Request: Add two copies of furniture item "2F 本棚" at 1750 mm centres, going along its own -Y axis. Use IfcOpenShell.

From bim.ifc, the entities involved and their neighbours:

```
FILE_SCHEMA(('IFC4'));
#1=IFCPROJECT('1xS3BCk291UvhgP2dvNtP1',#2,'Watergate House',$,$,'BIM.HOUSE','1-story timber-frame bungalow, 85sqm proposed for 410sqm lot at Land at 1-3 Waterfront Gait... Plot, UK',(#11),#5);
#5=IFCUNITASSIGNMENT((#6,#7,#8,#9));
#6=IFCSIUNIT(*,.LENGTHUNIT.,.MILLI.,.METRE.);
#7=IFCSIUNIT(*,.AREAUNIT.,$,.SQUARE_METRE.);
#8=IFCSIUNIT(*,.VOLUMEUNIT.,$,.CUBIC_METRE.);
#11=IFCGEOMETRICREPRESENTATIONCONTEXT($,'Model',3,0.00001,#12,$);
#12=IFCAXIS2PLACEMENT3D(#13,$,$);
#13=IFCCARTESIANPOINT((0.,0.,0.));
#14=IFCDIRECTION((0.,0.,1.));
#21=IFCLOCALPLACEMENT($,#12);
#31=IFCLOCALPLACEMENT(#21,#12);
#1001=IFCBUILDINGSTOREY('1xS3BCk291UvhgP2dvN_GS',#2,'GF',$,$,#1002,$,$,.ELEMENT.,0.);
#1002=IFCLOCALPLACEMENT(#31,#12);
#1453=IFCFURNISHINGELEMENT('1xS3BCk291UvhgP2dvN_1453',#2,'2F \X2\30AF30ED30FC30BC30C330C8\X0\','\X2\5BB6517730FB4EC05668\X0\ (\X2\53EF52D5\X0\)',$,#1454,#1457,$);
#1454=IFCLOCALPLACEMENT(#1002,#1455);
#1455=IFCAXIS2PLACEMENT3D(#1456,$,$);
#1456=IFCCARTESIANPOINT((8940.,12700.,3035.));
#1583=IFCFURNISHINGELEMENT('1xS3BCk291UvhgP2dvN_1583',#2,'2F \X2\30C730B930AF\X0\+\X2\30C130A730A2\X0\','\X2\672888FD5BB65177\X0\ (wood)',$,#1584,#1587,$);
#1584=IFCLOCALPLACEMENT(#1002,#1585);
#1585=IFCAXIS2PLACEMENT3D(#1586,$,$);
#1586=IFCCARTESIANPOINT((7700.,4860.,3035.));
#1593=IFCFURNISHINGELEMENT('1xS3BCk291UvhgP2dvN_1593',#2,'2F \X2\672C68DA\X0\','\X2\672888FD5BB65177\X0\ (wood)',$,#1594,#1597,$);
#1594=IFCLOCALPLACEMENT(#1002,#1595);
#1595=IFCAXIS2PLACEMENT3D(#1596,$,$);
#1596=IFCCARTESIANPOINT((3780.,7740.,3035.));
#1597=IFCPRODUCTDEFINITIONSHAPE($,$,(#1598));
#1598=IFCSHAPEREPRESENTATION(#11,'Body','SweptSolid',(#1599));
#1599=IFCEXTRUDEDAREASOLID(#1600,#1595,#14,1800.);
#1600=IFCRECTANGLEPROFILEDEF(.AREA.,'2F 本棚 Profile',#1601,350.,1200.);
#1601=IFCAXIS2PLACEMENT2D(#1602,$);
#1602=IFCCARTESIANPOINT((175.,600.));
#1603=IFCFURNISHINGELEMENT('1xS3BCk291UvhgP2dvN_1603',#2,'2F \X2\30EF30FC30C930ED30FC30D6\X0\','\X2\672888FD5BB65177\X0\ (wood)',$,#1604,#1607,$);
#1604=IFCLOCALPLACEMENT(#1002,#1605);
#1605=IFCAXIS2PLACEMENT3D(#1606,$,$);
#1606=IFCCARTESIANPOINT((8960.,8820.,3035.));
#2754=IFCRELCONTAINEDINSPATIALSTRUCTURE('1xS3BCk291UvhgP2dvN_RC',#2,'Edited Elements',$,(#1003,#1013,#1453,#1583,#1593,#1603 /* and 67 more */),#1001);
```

```python
import ifcopenshell
import ifcopenshell.api.geometry
import ifcopenshell.api.root
import ifcopenshell.util.element
import ifcopenshell.util.placement
import ifcopenshell.util.unit

model = ifcopenshell.open("bim.ifc")
unit_scale = ifcopenshell.util.unit.calculate_unit_scale(model)


def reuse_history(source, copy):
    """copy_class also copies each property set's owner history, people and application; keep the originals."""
    for rel in copy.IsDefinedBy:
        if rel.is_a("IfcRelDefinesByProperties") and (history := rel.RelatingPropertyDefinition.OwnerHistory):
            rel.RelatingPropertyDefinition.OwnerHistory = source.OwnerHistory
            ifcopenshell.util.element.remove_deep2(model, history)


source = model.by_guid("1xS3BCk291UvhgP2dvN_1593")
base = ifcopenshell.util.placement.get_local_placement(source.ObjectPlacement)
step = -base[:3, 1] * 1.75 / unit_scale

for i in range(1, 3):
    copy = ifcopenshell.api.root.copy_class(model, product=source)
    copy.Representation = ifcopenshell.util.element.copy_deep(
        model, source.Representation, exclude=["IfcGeometricRepresentationContext", "IfcRepresentationMap"]
    )
    reuse_history(source, copy)
    matrix = base.copy()
    matrix[:3, 3] += i * step
    print("added at", matrix[:3, 3].round(3) + 0.0)
    ifcopenshell.api.geometry.edit_object_placement(model, product=copy, matrix=matrix, is_si=False)

model.write("bim_v2.ifc")
```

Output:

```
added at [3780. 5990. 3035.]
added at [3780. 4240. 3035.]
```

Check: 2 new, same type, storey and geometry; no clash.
